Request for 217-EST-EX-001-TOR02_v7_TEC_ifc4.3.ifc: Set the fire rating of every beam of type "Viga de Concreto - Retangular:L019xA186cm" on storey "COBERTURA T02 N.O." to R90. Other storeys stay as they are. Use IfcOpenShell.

First a look at what the model holds.

```python
import ifcopenshell
import ifcopenshell.util.element

model = ifcopenshell.open("217-EST-EX-001-TOR02_v7_TEC_ifc4.3.ifc")
print(model.schema)
storey = next(s for s in model.by_type("IfcBuildingStorey") if s.Name == "COBERTURA T02 N.O.")
beams = [e for e in ifcopenshell.util.element.get_decomposition(storey) if e.is_a("IfcBeam")]
seen = {}
for e in beams:
    element_type = ifcopenshell.util.element.get_type(e)
    key = (element_type.Name if element_type != e and element_type else None, ifcopenshell.util.element.get_pset(e, "Pset_BeamCommon", "FireRating"))
    seen[key] = seen.get(key, 0) + 1
for (name, value), count in sorted(seen.items(), key=str):
    print(count, "x", name, "|", value)
```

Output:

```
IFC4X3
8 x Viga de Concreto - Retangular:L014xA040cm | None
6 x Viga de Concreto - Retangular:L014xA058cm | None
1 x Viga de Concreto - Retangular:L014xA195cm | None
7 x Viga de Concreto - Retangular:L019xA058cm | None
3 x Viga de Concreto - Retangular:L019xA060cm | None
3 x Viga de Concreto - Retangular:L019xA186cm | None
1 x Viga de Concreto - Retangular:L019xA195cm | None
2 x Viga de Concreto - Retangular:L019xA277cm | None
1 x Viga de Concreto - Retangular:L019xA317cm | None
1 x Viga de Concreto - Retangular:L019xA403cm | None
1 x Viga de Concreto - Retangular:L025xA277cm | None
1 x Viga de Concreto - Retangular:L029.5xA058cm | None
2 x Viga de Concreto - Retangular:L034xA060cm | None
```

```python
import ifcopenshell
import ifcopenshell.api.pset
import ifcopenshell.util.element

model = ifcopenshell.open("217-EST-EX-001-TOR02_v7_TEC_ifc4.3.ifc")

storey = next(s for s in model.by_type("IfcBuildingStorey") if s.Name == "COBERTURA T02 N.O.")
beams = [e for e in ifcopenshell.util.element.get_decomposition(storey) if e.is_a("IfcBeam")]

count = 0
for e in beams:
    element_type = ifcopenshell.util.element.get_type(e)
    if element_type in (None, e) or element_type.Name != "Viga de Concreto - Retangular:L019xA186cm":
        continue
    # add_pset returns the element's existing set when there is one.
    pset = ifcopenshell.api.pset.add_pset(model, product=e, name="Pset_BeamCommon")
    ifcopenshell.api.pset.edit_pset(model, pset=pset, properties={"FireRating": "R90"})
    count += 1

print(count, "beams updated")

model.write("217-EST-EX-001-TOR02_v7_TEC_ifc4.3_v2.ifc")
```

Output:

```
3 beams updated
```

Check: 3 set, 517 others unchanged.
